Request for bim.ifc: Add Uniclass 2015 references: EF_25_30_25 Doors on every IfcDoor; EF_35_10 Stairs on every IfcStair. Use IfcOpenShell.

First a look at what the model holds.

```python
import ifcopenshell

model = ifcopenshell.open("bim.ifc")
print(model.schema)
print("classifications:", [c.Name for c in model.by_type("IfcClassification")])
for ifc_class in ("IfcDoor", "IfcRoof", "IfcStair", "IfcWall", "IfcWindow"):
    print(ifc_class, len(model.by_type(ifc_class)))
```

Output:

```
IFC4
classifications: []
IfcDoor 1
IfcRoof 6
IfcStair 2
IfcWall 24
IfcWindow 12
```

```python
import ifcopenshell
import ifcopenshell.api.classification

model = ifcopenshell.open("bim.ifc")

system = ifcopenshell.api.classification.add_classification(model, classification="Uniclass 2015")

codes = {
    "IfcDoor": ("EF_25_30_25", "Doors"),
    "IfcStair": ("EF_35_10", "Stairs"),
}
for ifc_class, (code, name) in codes.items():
    products = model.by_type(ifc_class)
    ifcopenshell.api.classification.add_reference(
        model, products=products, classification=system, identification=code, name=name
    )
    print(code, len(products))

model.write("bim_updated.ifc")
```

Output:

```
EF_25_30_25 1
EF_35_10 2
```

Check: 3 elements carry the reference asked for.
